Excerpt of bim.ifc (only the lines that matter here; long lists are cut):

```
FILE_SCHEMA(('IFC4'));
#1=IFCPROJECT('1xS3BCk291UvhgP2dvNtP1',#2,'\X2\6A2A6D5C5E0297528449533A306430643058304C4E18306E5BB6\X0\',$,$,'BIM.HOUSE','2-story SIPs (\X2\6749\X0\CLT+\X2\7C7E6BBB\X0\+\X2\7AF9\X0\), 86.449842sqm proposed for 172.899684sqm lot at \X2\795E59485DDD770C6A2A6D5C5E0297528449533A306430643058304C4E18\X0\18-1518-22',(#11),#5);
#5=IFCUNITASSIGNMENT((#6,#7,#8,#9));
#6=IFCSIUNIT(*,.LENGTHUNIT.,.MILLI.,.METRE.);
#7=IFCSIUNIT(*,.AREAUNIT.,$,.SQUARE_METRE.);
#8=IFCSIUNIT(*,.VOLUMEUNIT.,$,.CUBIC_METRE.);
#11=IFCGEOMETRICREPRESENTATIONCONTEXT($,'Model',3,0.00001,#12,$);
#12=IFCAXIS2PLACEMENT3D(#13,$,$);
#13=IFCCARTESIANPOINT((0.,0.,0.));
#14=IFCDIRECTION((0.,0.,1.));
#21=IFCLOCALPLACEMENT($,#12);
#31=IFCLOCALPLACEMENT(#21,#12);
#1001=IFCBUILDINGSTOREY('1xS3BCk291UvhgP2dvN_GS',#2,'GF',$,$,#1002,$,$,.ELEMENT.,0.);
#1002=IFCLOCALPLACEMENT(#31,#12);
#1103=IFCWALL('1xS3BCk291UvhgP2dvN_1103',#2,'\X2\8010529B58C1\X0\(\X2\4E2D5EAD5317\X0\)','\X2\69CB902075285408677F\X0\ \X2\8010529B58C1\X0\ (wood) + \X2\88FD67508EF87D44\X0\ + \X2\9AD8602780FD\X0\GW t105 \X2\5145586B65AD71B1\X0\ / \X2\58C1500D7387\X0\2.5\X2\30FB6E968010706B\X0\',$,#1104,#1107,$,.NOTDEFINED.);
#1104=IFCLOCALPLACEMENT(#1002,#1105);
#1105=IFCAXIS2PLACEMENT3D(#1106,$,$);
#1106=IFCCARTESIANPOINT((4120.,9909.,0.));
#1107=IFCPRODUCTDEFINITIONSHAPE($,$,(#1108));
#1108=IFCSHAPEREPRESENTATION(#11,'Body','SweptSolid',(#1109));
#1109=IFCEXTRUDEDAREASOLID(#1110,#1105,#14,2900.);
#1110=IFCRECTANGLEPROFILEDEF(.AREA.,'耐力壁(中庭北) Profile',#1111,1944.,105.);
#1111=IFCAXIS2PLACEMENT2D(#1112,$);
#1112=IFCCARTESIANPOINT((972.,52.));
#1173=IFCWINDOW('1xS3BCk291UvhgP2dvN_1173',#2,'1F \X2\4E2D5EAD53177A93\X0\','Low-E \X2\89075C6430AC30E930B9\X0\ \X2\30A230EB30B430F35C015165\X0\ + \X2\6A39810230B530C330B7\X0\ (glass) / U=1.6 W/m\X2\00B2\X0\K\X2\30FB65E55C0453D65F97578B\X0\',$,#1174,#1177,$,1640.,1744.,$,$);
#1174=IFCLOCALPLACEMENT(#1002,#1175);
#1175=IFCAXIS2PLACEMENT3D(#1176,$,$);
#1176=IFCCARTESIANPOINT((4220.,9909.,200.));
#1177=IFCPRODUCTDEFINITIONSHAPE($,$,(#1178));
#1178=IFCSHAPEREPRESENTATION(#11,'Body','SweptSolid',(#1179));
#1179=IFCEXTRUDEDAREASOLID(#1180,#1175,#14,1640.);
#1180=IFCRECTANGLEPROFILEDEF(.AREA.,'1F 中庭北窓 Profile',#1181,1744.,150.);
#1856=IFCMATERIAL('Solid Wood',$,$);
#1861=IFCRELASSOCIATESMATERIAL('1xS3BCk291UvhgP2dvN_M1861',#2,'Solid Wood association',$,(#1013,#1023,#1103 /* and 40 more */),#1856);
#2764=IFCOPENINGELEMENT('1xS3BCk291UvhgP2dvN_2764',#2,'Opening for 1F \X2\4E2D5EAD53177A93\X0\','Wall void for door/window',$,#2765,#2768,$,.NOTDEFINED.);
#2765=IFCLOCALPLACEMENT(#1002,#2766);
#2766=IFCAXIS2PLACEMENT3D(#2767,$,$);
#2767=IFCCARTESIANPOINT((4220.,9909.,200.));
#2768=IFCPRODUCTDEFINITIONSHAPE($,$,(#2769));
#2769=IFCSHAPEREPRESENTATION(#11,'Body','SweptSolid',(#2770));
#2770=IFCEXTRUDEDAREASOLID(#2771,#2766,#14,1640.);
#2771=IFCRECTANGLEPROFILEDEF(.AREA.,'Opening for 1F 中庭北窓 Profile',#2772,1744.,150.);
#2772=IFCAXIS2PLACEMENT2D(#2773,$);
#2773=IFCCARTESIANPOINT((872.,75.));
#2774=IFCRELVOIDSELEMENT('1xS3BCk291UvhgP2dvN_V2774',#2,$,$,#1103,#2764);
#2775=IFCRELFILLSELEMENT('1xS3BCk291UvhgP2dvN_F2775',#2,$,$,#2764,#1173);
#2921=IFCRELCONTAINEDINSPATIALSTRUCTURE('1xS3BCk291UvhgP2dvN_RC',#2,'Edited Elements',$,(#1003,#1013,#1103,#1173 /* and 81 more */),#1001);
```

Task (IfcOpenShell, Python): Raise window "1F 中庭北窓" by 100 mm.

```python
import numpy as np
import ifcopenshell
import ifcopenshell.api.geometry
import ifcopenshell.util.placement
import ifcopenshell.util.unit

model = ifcopenshell.open("bim.ifc")
unit_scale = ifcopenshell.util.unit.calculate_unit_scale(model)

window = model.by_guid("1xS3BCk291UvhgP2dvN_1173")
opening = window.FillsVoids[0].RelatingOpeningElement
dz = 100.0

shift = np.array([0.0, 0.0, dz])
# The window is not placed relative to its opening, so move both.
for product in (opening, window):
    matrix = ifcopenshell.util.placement.get_local_placement(product.ObjectPlacement)
    matrix[:3, 3] += shift
    ifcopenshell.api.geometry.edit_object_placement(model, product=product, matrix=matrix, is_si=False)

print(f"moved by {dz * unit_scale:+.3f} m")

model.write("bim_rev.ifc")
```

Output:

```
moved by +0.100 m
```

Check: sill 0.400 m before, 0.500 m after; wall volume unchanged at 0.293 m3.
